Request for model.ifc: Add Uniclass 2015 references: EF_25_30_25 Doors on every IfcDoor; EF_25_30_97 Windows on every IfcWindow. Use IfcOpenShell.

First a look at what the model holds.

```python
import ifcopenshell

model = ifcopenshell.open("model.ifc")
print(model.schema)
print("classifications:", [c.Name for c in model.by_type("IfcClassification")])
for ifc_class in ("IfcDoor", "IfcRoof", "IfcStair", "IfcWall", "IfcWindow"):
    print(ifc_class, len(model.by_type(ifc_class)))
```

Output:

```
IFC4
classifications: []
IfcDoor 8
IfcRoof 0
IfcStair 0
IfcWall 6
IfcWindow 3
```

```python
import ifcopenshell
import ifcopenshell.api.classification

model = ifcopenshell.open("model.ifc")

system = ifcopenshell.api.classification.add_classification(model, classification="Uniclass 2015")

codes = {
    "IfcDoor": ("EF_25_30_25", "Doors"),
    "IfcWindow": ("EF_25_30_97", "Windows"),
}
for ifc_class, (code, name) in codes.items():
    products = model.by_type(ifc_class)
    ifcopenshell.api.classification.add_reference(
        model, products=products, classification=system, identification=code, name=name
    )
    print(code, len(products))

model.write("model-out.ifc")
```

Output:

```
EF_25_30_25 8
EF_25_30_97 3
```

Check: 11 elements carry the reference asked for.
